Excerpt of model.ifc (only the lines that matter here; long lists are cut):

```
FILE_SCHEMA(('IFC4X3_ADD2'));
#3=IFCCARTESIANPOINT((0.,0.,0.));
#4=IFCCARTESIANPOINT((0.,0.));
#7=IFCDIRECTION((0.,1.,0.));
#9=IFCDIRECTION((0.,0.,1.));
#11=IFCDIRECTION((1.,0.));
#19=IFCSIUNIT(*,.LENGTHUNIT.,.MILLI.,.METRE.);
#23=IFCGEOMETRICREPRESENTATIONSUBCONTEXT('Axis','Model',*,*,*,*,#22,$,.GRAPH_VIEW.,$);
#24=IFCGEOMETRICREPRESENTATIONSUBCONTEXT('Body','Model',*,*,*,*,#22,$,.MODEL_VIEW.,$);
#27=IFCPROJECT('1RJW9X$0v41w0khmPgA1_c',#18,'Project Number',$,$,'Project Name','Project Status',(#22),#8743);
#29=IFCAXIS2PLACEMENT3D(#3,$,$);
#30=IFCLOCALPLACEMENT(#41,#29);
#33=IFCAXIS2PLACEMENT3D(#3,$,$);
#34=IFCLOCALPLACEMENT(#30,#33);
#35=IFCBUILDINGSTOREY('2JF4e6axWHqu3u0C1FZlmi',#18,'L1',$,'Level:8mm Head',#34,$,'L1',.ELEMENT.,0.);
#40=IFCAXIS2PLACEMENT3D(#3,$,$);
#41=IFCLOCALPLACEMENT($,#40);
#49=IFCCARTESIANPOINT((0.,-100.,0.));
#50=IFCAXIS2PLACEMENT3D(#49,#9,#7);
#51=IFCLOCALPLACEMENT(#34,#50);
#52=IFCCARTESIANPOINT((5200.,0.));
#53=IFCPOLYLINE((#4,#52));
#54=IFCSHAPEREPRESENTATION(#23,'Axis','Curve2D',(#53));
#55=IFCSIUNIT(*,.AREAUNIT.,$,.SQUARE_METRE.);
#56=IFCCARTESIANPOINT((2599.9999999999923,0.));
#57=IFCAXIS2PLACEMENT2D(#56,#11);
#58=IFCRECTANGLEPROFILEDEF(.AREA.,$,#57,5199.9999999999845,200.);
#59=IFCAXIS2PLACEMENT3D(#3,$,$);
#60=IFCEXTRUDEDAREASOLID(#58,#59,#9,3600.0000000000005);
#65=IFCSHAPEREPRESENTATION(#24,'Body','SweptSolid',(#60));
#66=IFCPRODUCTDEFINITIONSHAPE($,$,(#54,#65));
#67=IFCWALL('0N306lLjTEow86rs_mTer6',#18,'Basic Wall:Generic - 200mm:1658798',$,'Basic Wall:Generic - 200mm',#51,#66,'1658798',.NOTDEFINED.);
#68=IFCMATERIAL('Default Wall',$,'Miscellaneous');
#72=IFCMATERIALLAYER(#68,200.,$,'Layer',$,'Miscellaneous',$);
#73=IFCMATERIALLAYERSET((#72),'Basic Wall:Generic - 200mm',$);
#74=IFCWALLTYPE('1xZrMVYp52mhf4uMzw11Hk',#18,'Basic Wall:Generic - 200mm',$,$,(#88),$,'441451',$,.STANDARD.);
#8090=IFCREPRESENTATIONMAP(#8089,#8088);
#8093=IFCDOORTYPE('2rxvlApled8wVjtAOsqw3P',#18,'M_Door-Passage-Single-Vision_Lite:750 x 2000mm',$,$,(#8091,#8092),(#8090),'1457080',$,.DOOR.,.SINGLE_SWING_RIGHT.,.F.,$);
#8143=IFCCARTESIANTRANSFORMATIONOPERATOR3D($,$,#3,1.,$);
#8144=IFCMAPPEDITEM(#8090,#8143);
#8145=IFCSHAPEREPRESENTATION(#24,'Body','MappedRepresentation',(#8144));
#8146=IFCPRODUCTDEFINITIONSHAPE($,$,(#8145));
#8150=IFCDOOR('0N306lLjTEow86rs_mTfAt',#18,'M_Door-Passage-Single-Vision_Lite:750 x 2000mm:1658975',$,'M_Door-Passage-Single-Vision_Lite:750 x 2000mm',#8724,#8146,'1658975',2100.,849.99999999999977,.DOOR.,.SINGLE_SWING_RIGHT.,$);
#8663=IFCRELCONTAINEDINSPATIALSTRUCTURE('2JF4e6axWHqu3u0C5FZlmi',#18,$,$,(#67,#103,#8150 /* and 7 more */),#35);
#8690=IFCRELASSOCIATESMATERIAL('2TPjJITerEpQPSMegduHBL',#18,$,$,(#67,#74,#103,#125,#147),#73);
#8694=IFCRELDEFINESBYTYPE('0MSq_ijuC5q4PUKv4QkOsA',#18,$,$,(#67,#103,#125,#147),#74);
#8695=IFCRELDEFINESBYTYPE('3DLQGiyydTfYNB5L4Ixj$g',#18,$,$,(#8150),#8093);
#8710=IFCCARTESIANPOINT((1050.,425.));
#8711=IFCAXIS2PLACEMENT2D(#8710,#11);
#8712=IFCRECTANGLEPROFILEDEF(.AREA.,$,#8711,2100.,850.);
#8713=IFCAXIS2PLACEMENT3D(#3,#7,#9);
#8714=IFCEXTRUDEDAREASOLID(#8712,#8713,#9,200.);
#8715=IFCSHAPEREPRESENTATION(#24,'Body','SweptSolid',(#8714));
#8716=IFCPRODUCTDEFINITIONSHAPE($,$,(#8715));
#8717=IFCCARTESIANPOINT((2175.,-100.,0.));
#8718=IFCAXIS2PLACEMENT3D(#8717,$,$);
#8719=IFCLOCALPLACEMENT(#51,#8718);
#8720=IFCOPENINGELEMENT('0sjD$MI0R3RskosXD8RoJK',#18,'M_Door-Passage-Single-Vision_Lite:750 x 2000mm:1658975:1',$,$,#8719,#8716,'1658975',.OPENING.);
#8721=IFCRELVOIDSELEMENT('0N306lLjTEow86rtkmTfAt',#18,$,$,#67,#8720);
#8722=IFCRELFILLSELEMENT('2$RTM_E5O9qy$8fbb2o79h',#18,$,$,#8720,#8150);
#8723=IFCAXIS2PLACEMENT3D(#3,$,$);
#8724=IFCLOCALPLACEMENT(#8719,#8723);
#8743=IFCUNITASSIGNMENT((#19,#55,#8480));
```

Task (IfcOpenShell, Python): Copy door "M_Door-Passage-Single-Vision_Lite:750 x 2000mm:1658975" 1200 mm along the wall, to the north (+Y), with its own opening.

```python
import ifcopenshell
import ifcopenshell.api.feature
import ifcopenshell.api.geometry
import ifcopenshell.api.root
import ifcopenshell.geom
import ifcopenshell.util.element
import ifcopenshell.util.placement
import ifcopenshell.util.shape
import ifcopenshell.util.unit

model = ifcopenshell.open("model.ifc")
unit_scale = ifcopenshell.util.unit.calculate_unit_scale(model)
settings = ifcopenshell.geom.settings()


def volume(element):
    """Net volume in cubic metres, openings subtracted."""
    shape = ifcopenshell.geom.create_shape(settings, element)
    return ifcopenshell.util.shape.get_volume(shape.geometry)


def reuse_history(source, copy):
    """copy_class also copies each property set's owner history, people and application; keep the originals."""
    for rel in copy.IsDefinedBy:
        if rel.is_a("IfcRelDefinesByProperties") and (history := rel.RelatingPropertyDefinition.OwnerHistory):
            rel.RelatingPropertyDefinition.OwnerHistory = source.OwnerHistory
            ifcopenshell.util.element.remove_deep2(model, history)


door = model.by_guid("0N306lLjTEow86rs_mTfAt")
opening = door.FillsVoids[0].RelatingOpeningElement
wall = opening.VoidsElements[0].RelatingBuildingElement
before = volume(wall)
shift = ifcopenshell.util.placement.get_local_placement(wall.ObjectPlacement)[:3, 0] * 1.2 / unit_scale

# copy_class copies the void relationship, type, container and properties, but no geometry.
new_opening = ifcopenshell.api.root.copy_class(model, product=opening)
new_opening.Representation = ifcopenshell.util.element.copy_deep(
    model, opening.Representation, exclude=["IfcGeometricRepresentationContext", "IfcRepresentationMap"]
)
new_opening.Name = "M_Door-Passage-Single-Vision_Lite:750 x 2000mm"
new_opening.Tag = None
new_door = ifcopenshell.api.root.copy_class(model, product=door)
new_door.Representation = ifcopenshell.util.element.copy_deep(
    model, door.Representation, exclude=["IfcGeometricRepresentationContext", "IfcRepresentationMap"]
)
new_door.Name = "M_Door-Passage-Single-Vision_Lite:750 x 2000mm"
new_door.Tag = None
reuse_history(door, new_door)
ifcopenshell.api.feature.add_filling(model, opening=new_opening, element=new_door)

for old, new in ((opening, new_opening), (door, new_door)):
    matrix = ifcopenshell.util.placement.get_local_placement(old.ObjectPlacement)
    matrix[:3, 3] += shift
    ifcopenshell.api.geometry.edit_object_placement(model, product=new, matrix=matrix, is_si=False)

after = volume(wall)

print(f"wall volume {before:.3f} -> {after:.3f} m3")

model.write("model_edited.ifc")
```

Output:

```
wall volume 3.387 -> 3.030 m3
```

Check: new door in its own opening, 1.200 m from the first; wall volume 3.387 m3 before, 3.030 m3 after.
